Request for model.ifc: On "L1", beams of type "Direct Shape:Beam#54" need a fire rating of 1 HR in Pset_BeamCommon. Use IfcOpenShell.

First a look at what the model holds.

```python
import ifcopenshell
import ifcopenshell.util.element

model = ifcopenshell.open("model.ifc")
print(model.schema)
storey = next(s for s in model.by_type("IfcBuildingStorey") if s.Name == "L1")
beams = [e for e in ifcopenshell.util.element.get_decomposition(storey) if e.is_a("IfcBeam")]
seen = {}
for e in beams:
    element_type = ifcopenshell.util.element.get_type(e)
    key = (element_type.Name if element_type != e and element_type else None, ifcopenshell.util.element.get_pset(e, "Pset_BeamCommon", "FireRating"))
    seen[key] = seen.get(key, 0) + 1
for (name, value), count in sorted(seen.items(), key=str):
    print(count, "x", name, "|", value)
```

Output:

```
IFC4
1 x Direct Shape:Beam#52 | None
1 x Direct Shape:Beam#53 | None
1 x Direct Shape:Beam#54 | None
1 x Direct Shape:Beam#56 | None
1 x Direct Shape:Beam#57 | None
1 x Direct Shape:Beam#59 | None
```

```python
import ifcopenshell
import ifcopenshell.api.pset
import ifcopenshell.util.element

model = ifcopenshell.open("model.ifc")

storey = next(s for s in model.by_type("IfcBuildingStorey") if s.Name == "L1")
beams = [e for e in ifcopenshell.util.element.get_decomposition(storey) if e.is_a("IfcBeam")]

count = 0
for e in beams:
    element_type = ifcopenshell.util.element.get_type(e)
    if element_type in (None, e) or element_type.Name != "Direct Shape:Beam#54":
        continue
    # add_pset returns the element's existing set when there is one.
    pset = ifcopenshell.api.pset.add_pset(model, product=e, name="Pset_BeamCommon")
    ifcopenshell.api.pset.edit_pset(model, pset=pset, properties={"FireRating": "1 HR"})
    count += 1

print(count, "beams updated")

model.write("model_rev.ifc")
```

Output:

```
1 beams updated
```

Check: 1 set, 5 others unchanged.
